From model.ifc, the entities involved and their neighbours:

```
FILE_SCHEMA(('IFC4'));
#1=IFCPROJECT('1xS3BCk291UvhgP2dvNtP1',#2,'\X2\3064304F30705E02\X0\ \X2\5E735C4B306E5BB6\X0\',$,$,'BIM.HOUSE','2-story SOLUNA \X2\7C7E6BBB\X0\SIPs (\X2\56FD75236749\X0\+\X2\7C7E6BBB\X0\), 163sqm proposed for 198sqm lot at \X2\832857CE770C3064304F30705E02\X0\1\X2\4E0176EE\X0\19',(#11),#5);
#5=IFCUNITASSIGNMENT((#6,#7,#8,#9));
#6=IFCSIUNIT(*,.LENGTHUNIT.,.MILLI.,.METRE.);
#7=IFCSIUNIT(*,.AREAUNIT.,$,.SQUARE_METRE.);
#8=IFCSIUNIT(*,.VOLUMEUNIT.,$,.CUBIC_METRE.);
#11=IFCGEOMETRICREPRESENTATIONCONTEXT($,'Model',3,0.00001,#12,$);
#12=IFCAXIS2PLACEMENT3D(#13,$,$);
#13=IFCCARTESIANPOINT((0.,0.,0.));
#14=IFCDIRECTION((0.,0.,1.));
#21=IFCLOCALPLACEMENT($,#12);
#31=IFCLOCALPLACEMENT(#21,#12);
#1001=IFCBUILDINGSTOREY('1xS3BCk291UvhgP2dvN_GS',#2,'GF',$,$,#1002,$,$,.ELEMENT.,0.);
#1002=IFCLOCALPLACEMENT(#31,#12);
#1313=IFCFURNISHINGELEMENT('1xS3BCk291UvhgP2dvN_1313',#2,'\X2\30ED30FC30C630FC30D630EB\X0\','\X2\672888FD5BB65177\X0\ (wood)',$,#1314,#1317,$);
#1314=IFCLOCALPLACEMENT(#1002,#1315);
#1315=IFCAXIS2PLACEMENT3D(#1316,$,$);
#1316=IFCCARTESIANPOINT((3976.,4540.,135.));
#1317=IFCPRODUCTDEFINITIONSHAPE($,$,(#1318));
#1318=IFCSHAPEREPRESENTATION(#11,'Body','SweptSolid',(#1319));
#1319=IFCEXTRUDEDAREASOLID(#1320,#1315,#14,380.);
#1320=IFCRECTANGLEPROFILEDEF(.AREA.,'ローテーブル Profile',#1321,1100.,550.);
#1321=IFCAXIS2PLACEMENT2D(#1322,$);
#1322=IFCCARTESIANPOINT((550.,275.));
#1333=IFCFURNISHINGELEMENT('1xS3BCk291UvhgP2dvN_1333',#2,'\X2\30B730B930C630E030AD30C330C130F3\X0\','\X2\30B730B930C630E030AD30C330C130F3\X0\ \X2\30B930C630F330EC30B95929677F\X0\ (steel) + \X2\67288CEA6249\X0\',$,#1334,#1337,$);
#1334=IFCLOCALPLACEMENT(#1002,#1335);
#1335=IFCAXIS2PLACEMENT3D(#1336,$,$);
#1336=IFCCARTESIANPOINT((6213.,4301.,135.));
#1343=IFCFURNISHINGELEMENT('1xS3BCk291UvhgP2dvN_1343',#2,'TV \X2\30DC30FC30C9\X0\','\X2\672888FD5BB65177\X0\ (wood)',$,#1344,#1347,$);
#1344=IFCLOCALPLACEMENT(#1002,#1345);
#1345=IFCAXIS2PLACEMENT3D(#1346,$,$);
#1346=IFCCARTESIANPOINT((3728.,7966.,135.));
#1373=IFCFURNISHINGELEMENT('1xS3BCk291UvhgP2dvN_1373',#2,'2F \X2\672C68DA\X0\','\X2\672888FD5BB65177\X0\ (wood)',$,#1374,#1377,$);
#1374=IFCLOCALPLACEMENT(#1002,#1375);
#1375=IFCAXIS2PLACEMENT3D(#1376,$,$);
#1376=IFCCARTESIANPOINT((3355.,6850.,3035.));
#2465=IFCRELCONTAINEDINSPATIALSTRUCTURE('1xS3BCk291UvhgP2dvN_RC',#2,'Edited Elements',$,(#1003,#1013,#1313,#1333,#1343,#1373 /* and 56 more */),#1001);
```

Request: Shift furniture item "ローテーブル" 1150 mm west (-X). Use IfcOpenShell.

```python
import ifcopenshell
import ifcopenshell.api.geometry
import ifcopenshell.util.placement

model = ifcopenshell.open("model.ifc")

item = model.by_guid("1xS3BCk291UvhgP2dvN_1313")
matrix = ifcopenshell.util.placement.get_local_placement(item.ObjectPlacement)
matrix[0, 3] -= 1150.0
ifcopenshell.api.geometry.edit_object_placement(model, product=item, matrix=matrix, is_si=False)

print(ifcopenshell.util.placement.get_local_placement(item.ObjectPlacement).round(3) + 0.0)

model.write("model_updated.ifc")
```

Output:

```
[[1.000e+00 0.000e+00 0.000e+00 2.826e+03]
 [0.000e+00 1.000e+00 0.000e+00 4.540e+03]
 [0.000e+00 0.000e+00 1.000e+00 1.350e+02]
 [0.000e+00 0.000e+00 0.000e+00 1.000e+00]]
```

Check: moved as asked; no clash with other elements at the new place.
